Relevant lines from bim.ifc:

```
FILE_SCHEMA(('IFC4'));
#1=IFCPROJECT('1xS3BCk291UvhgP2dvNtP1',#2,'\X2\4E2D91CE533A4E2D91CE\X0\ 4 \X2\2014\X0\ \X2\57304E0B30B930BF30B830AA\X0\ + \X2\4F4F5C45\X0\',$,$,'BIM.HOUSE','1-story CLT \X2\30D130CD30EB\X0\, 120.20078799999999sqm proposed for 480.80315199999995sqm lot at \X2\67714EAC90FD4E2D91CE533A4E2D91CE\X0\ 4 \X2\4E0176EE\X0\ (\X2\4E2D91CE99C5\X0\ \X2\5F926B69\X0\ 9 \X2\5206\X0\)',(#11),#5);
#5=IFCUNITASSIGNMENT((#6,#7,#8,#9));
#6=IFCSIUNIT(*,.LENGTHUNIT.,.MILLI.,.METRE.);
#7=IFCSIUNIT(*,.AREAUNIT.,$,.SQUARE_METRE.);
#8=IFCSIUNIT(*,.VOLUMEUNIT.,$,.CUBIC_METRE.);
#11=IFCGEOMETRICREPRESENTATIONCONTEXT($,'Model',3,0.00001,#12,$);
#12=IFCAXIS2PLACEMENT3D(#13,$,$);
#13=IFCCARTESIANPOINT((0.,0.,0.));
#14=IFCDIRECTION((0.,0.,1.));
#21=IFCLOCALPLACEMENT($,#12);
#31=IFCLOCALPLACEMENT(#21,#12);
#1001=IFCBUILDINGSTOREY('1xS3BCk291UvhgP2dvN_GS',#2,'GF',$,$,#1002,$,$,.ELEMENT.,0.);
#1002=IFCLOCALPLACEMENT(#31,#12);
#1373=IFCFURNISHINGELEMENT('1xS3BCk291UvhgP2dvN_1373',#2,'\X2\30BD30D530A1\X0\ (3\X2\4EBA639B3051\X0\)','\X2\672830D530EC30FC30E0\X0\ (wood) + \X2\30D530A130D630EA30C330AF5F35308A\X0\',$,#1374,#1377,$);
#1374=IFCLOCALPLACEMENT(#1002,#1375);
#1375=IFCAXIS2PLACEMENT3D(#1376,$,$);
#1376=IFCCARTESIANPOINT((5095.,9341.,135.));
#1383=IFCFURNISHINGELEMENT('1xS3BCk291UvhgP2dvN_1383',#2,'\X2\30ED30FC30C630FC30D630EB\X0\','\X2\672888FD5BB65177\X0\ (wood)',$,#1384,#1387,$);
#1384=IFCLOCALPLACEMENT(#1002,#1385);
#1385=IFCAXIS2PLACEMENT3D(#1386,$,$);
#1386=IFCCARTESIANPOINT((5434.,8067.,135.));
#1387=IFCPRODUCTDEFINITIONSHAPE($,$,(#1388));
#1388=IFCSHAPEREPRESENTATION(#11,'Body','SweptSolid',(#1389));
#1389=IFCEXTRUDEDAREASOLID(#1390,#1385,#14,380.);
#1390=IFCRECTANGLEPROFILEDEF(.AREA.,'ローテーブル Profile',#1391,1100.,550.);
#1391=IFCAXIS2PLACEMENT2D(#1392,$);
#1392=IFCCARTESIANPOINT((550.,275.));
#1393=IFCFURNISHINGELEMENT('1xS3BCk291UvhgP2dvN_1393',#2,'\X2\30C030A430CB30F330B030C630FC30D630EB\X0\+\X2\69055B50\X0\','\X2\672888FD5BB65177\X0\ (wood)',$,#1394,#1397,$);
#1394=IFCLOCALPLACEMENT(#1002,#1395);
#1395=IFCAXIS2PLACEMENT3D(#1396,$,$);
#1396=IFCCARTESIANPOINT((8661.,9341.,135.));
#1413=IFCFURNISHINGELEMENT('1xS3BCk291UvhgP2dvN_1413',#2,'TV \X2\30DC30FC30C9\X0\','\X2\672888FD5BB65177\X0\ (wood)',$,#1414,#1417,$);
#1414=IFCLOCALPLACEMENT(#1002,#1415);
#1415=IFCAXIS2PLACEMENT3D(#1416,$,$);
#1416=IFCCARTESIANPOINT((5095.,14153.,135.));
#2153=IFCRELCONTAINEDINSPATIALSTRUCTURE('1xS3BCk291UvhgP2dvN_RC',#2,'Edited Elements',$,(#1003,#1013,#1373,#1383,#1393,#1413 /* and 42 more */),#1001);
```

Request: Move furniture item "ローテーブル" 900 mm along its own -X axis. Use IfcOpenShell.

```python
import ifcopenshell
import ifcopenshell.api.geometry
import ifcopenshell.util.placement
import ifcopenshell.util.unit

model = ifcopenshell.open("bim.ifc")
unit_scale = ifcopenshell.util.unit.calculate_unit_scale(model)

item = model.by_guid("1xS3BCk291UvhgP2dvN_1383")
matrix = ifcopenshell.util.placement.get_local_placement(item.ObjectPlacement)
matrix[:3, 3] -= matrix[:3, 0] * 0.9 / unit_scale
ifcopenshell.api.geometry.edit_object_placement(model, product=item, matrix=matrix, is_si=False)

print(ifcopenshell.util.placement.get_local_placement(item.ObjectPlacement).round(3) + 0.0)

model.write("bim_updated.ifc")
```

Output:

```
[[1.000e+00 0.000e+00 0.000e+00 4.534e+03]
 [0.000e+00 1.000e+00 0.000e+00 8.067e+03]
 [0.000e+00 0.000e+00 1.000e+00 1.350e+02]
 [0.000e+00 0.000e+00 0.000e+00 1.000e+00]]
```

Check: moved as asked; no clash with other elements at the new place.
